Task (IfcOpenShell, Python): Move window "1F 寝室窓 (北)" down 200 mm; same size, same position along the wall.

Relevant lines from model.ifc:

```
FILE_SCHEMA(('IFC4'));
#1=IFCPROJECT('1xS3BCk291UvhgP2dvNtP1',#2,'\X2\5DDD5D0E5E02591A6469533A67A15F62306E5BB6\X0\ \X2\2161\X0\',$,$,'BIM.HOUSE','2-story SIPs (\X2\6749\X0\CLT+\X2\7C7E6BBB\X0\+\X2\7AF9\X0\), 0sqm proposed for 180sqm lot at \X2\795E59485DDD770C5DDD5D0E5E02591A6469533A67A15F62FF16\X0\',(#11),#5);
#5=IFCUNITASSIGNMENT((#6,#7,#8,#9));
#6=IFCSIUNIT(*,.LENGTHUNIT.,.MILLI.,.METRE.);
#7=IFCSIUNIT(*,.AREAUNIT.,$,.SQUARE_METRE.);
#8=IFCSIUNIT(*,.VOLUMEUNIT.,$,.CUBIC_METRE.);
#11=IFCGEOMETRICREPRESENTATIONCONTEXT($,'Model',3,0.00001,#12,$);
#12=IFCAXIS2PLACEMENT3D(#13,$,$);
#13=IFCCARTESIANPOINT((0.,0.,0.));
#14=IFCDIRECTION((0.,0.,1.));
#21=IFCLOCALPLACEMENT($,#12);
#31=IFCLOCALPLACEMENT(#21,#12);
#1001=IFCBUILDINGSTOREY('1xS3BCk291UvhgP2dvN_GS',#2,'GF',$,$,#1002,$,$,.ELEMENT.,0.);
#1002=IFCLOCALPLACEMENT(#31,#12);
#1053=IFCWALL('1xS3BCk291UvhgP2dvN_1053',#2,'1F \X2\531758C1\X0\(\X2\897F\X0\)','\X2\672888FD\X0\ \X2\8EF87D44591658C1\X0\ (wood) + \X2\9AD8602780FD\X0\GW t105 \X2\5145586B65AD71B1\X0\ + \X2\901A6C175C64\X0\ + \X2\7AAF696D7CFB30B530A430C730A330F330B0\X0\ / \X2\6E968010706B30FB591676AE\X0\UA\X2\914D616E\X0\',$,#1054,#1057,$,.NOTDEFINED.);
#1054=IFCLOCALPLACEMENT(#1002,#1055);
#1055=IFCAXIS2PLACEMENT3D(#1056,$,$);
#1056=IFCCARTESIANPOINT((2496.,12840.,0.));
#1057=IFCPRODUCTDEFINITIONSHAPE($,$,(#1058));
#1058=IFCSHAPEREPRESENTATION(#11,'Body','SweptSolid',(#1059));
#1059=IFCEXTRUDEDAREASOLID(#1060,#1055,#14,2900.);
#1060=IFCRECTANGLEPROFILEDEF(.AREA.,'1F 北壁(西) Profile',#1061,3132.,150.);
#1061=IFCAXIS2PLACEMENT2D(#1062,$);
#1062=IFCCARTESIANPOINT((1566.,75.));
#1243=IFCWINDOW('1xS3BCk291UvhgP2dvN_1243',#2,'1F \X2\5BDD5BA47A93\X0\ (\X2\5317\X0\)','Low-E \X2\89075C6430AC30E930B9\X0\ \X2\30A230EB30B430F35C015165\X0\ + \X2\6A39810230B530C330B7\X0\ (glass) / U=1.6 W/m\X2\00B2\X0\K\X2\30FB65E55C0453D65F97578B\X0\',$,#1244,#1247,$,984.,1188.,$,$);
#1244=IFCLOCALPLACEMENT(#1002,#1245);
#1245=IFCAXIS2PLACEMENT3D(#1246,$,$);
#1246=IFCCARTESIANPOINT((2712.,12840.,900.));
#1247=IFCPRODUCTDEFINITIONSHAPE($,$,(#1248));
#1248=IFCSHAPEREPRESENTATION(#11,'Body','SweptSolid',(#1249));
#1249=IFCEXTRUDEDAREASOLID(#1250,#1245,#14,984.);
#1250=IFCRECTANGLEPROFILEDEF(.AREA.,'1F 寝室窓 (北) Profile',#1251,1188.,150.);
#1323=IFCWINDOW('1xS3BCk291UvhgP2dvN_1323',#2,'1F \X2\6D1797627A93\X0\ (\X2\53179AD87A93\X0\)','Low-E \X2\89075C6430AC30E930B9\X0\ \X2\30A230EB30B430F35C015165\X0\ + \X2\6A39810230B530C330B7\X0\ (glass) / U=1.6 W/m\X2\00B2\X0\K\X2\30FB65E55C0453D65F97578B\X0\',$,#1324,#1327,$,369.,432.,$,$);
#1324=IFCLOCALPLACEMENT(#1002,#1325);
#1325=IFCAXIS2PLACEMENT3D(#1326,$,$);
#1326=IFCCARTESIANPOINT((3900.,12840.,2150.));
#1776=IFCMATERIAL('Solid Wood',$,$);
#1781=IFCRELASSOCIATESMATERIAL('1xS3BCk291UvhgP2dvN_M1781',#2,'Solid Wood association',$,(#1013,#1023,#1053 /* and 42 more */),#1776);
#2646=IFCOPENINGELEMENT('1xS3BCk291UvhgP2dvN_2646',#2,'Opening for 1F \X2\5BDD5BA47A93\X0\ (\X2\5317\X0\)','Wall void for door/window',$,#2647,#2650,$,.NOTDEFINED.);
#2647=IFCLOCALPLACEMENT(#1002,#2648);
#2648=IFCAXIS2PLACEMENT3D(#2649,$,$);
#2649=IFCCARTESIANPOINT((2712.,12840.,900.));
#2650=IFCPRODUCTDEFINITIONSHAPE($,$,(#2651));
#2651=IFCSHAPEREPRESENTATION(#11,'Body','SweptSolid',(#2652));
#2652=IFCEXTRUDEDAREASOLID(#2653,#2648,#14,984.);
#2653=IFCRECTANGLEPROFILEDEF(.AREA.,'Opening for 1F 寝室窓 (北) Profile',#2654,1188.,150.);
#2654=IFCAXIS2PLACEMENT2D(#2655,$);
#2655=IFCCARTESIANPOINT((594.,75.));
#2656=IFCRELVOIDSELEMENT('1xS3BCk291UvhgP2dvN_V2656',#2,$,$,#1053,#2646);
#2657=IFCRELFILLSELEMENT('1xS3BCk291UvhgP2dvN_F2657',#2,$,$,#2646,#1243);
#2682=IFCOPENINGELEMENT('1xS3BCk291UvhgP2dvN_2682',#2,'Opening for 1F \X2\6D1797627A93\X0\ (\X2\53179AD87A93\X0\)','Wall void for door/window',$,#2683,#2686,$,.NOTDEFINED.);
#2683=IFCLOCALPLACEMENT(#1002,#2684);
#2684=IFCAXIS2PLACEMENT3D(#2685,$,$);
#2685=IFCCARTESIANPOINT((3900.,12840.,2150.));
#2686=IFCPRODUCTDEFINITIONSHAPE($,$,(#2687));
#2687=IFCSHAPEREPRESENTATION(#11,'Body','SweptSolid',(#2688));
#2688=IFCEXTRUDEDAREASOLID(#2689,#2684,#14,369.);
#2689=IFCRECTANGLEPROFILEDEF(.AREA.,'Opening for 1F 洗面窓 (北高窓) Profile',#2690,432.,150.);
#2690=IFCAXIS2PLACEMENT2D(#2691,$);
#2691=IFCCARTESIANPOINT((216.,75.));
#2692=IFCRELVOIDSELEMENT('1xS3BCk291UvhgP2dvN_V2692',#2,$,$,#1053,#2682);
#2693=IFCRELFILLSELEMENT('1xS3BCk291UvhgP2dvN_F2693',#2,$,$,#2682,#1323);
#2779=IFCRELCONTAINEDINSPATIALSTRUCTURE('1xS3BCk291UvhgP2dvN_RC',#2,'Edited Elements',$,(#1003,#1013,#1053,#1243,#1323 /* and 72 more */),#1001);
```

```python
import numpy as np
import ifcopenshell
import ifcopenshell.api.geometry
import ifcopenshell.util.placement
import ifcopenshell.util.unit

model = ifcopenshell.open("model.ifc")
unit_scale = ifcopenshell.util.unit.calculate_unit_scale(model)

window = model.by_guid("1xS3BCk291UvhgP2dvN_1243")
opening = window.FillsVoids[0].RelatingOpeningElement
dz = -200.0

shift = np.array([0.0, 0.0, dz])
# The window is not placed relative to its opening, so move both.
for product in (opening, window):
    matrix = ifcopenshell.util.placement.get_local_placement(product.ObjectPlacement)
    matrix[:3, 3] += shift
    ifcopenshell.api.geometry.edit_object_placement(model, product=product, matrix=matrix, is_si=False)

print(f"moved by {dz * unit_scale:+.3f} m")

model.write("model_updated.ifc")
```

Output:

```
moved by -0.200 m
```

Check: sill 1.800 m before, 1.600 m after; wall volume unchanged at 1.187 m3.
